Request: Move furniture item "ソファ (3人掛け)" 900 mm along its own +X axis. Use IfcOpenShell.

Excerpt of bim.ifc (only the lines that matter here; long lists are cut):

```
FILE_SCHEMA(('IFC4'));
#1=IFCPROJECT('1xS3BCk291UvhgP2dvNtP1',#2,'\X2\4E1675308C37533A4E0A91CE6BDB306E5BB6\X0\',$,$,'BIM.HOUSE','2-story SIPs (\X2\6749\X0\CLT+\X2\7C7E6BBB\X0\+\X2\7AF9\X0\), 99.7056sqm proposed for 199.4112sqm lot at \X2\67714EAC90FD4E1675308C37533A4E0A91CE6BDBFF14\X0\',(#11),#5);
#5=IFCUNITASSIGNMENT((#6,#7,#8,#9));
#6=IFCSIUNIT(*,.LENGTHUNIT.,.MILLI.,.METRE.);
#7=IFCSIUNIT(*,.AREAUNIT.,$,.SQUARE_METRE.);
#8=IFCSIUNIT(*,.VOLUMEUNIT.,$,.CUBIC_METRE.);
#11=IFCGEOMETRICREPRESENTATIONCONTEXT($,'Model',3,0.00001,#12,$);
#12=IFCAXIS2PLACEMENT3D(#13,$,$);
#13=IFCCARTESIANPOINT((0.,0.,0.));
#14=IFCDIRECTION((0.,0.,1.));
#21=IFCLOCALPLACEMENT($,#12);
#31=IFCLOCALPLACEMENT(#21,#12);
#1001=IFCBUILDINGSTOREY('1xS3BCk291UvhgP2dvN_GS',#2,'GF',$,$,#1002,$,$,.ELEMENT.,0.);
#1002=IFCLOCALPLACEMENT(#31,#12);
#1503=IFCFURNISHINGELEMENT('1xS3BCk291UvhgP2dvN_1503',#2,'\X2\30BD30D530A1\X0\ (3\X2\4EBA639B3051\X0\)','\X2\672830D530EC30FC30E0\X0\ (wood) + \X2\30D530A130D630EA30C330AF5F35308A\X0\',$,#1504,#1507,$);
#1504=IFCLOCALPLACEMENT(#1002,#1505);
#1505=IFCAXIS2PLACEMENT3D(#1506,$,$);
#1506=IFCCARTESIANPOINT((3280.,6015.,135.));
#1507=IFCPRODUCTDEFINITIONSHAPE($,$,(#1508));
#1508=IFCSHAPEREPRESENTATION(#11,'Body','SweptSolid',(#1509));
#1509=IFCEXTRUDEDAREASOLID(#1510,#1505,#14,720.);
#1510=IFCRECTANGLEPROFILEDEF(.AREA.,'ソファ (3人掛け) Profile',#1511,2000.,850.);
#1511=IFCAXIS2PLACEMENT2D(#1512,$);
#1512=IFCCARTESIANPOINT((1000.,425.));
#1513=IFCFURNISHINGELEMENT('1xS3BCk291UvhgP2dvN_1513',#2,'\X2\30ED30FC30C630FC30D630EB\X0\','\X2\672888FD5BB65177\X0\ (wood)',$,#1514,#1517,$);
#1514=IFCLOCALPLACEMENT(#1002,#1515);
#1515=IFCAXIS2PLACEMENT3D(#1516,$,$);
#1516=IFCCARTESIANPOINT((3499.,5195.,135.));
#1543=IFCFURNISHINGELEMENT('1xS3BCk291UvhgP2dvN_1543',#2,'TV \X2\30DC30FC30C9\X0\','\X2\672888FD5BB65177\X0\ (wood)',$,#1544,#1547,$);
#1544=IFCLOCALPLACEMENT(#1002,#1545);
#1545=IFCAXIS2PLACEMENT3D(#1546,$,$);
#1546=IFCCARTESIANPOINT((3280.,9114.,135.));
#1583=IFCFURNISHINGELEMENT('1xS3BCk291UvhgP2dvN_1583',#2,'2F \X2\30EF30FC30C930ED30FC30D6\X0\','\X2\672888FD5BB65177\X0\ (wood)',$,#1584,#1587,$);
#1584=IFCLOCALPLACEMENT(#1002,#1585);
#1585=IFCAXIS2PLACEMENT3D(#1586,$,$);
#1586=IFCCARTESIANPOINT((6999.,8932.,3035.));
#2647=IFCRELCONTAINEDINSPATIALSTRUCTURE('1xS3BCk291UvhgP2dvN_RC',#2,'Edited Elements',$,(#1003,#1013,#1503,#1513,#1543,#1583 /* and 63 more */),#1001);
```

```python
import ifcopenshell
import ifcopenshell.api.geometry
import ifcopenshell.util.placement

model = ifcopenshell.open("bim.ifc")

item = model.by_guid("1xS3BCk291UvhgP2dvN_1503")
matrix = ifcopenshell.util.placement.get_local_placement(item.ObjectPlacement)
matrix[:3, 3] += matrix[:3, 0] * 900.0
ifcopenshell.api.geometry.edit_object_placement(model, product=item, matrix=matrix, is_si=False)

print(ifcopenshell.util.placement.get_local_placement(item.ObjectPlacement).round(3) + 0.0)

model.write("bim_rev.ifc")
```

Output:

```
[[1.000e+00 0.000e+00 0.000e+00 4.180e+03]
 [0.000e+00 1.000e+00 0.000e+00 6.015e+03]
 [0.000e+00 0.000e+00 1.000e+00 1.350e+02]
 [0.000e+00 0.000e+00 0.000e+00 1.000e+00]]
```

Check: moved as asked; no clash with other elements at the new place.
